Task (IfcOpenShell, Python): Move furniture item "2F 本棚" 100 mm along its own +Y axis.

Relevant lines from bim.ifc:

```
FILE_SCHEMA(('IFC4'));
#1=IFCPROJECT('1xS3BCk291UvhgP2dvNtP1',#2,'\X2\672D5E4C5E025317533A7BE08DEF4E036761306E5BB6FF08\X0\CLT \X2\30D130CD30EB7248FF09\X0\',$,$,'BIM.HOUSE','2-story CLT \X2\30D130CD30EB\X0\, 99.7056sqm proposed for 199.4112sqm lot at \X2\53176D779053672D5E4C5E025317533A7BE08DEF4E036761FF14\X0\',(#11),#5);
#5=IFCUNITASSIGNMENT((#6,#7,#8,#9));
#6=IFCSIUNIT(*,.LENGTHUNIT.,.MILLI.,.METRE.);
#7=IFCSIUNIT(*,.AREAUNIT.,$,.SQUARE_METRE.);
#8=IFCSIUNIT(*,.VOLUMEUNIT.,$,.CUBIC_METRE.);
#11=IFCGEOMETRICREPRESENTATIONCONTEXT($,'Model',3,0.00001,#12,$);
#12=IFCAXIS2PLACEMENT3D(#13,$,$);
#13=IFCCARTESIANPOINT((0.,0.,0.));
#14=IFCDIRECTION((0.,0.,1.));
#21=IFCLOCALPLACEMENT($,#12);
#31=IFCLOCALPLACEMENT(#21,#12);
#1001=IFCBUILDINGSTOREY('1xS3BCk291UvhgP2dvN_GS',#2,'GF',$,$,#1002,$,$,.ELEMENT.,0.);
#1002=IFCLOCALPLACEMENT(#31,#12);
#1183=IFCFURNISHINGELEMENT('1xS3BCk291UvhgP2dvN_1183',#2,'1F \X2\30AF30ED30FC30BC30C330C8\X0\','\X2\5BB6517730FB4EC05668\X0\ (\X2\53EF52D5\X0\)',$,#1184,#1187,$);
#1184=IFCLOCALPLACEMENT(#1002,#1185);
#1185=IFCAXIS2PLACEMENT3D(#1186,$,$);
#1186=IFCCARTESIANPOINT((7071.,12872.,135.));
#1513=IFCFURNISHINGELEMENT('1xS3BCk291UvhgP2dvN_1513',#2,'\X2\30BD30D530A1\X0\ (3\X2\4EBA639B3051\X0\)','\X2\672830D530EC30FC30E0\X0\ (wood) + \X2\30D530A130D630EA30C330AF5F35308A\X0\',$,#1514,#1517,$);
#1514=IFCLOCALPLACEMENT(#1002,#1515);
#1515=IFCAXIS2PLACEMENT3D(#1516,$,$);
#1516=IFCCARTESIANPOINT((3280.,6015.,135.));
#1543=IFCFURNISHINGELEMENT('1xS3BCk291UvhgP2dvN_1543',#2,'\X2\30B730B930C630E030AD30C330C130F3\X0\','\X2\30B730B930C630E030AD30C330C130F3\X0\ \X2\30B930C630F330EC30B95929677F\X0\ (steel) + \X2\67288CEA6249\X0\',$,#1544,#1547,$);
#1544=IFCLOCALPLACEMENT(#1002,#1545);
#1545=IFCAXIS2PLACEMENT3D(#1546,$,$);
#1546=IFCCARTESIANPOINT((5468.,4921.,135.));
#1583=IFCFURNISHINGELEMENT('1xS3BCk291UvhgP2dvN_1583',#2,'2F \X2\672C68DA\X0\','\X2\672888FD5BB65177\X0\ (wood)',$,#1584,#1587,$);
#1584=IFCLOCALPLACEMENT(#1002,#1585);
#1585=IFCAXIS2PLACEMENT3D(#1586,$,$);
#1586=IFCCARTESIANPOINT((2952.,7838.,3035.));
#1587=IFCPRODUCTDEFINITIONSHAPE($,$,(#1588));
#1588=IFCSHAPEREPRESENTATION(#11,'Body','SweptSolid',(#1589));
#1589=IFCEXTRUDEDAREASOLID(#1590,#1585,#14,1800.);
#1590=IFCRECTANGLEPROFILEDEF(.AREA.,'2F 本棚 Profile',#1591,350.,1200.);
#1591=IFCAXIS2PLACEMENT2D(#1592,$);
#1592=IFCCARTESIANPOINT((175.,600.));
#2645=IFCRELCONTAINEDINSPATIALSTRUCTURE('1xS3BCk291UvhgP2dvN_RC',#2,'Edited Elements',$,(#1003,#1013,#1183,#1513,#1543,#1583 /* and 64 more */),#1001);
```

```python
import ifcopenshell
import ifcopenshell.api.geometry
import ifcopenshell.util.placement
import ifcopenshell.util.unit

model = ifcopenshell.open("bim.ifc")
unit_scale = ifcopenshell.util.unit.calculate_unit_scale(model)

item = model.by_guid("1xS3BCk291UvhgP2dvN_1583")
matrix = ifcopenshell.util.placement.get_local_placement(item.ObjectPlacement)
matrix[:3, 3] += matrix[:3, 1] * 0.1 / unit_scale
ifcopenshell.api.geometry.edit_object_placement(model, product=item, matrix=matrix, is_si=False)

print(ifcopenshell.util.placement.get_local_placement(item.ObjectPlacement).round(3) + 0.0)

model.write("bim_v2.ifc")
```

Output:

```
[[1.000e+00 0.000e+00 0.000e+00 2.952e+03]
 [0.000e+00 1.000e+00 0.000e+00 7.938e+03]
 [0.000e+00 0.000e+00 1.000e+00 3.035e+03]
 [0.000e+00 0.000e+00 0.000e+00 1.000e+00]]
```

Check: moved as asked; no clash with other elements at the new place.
